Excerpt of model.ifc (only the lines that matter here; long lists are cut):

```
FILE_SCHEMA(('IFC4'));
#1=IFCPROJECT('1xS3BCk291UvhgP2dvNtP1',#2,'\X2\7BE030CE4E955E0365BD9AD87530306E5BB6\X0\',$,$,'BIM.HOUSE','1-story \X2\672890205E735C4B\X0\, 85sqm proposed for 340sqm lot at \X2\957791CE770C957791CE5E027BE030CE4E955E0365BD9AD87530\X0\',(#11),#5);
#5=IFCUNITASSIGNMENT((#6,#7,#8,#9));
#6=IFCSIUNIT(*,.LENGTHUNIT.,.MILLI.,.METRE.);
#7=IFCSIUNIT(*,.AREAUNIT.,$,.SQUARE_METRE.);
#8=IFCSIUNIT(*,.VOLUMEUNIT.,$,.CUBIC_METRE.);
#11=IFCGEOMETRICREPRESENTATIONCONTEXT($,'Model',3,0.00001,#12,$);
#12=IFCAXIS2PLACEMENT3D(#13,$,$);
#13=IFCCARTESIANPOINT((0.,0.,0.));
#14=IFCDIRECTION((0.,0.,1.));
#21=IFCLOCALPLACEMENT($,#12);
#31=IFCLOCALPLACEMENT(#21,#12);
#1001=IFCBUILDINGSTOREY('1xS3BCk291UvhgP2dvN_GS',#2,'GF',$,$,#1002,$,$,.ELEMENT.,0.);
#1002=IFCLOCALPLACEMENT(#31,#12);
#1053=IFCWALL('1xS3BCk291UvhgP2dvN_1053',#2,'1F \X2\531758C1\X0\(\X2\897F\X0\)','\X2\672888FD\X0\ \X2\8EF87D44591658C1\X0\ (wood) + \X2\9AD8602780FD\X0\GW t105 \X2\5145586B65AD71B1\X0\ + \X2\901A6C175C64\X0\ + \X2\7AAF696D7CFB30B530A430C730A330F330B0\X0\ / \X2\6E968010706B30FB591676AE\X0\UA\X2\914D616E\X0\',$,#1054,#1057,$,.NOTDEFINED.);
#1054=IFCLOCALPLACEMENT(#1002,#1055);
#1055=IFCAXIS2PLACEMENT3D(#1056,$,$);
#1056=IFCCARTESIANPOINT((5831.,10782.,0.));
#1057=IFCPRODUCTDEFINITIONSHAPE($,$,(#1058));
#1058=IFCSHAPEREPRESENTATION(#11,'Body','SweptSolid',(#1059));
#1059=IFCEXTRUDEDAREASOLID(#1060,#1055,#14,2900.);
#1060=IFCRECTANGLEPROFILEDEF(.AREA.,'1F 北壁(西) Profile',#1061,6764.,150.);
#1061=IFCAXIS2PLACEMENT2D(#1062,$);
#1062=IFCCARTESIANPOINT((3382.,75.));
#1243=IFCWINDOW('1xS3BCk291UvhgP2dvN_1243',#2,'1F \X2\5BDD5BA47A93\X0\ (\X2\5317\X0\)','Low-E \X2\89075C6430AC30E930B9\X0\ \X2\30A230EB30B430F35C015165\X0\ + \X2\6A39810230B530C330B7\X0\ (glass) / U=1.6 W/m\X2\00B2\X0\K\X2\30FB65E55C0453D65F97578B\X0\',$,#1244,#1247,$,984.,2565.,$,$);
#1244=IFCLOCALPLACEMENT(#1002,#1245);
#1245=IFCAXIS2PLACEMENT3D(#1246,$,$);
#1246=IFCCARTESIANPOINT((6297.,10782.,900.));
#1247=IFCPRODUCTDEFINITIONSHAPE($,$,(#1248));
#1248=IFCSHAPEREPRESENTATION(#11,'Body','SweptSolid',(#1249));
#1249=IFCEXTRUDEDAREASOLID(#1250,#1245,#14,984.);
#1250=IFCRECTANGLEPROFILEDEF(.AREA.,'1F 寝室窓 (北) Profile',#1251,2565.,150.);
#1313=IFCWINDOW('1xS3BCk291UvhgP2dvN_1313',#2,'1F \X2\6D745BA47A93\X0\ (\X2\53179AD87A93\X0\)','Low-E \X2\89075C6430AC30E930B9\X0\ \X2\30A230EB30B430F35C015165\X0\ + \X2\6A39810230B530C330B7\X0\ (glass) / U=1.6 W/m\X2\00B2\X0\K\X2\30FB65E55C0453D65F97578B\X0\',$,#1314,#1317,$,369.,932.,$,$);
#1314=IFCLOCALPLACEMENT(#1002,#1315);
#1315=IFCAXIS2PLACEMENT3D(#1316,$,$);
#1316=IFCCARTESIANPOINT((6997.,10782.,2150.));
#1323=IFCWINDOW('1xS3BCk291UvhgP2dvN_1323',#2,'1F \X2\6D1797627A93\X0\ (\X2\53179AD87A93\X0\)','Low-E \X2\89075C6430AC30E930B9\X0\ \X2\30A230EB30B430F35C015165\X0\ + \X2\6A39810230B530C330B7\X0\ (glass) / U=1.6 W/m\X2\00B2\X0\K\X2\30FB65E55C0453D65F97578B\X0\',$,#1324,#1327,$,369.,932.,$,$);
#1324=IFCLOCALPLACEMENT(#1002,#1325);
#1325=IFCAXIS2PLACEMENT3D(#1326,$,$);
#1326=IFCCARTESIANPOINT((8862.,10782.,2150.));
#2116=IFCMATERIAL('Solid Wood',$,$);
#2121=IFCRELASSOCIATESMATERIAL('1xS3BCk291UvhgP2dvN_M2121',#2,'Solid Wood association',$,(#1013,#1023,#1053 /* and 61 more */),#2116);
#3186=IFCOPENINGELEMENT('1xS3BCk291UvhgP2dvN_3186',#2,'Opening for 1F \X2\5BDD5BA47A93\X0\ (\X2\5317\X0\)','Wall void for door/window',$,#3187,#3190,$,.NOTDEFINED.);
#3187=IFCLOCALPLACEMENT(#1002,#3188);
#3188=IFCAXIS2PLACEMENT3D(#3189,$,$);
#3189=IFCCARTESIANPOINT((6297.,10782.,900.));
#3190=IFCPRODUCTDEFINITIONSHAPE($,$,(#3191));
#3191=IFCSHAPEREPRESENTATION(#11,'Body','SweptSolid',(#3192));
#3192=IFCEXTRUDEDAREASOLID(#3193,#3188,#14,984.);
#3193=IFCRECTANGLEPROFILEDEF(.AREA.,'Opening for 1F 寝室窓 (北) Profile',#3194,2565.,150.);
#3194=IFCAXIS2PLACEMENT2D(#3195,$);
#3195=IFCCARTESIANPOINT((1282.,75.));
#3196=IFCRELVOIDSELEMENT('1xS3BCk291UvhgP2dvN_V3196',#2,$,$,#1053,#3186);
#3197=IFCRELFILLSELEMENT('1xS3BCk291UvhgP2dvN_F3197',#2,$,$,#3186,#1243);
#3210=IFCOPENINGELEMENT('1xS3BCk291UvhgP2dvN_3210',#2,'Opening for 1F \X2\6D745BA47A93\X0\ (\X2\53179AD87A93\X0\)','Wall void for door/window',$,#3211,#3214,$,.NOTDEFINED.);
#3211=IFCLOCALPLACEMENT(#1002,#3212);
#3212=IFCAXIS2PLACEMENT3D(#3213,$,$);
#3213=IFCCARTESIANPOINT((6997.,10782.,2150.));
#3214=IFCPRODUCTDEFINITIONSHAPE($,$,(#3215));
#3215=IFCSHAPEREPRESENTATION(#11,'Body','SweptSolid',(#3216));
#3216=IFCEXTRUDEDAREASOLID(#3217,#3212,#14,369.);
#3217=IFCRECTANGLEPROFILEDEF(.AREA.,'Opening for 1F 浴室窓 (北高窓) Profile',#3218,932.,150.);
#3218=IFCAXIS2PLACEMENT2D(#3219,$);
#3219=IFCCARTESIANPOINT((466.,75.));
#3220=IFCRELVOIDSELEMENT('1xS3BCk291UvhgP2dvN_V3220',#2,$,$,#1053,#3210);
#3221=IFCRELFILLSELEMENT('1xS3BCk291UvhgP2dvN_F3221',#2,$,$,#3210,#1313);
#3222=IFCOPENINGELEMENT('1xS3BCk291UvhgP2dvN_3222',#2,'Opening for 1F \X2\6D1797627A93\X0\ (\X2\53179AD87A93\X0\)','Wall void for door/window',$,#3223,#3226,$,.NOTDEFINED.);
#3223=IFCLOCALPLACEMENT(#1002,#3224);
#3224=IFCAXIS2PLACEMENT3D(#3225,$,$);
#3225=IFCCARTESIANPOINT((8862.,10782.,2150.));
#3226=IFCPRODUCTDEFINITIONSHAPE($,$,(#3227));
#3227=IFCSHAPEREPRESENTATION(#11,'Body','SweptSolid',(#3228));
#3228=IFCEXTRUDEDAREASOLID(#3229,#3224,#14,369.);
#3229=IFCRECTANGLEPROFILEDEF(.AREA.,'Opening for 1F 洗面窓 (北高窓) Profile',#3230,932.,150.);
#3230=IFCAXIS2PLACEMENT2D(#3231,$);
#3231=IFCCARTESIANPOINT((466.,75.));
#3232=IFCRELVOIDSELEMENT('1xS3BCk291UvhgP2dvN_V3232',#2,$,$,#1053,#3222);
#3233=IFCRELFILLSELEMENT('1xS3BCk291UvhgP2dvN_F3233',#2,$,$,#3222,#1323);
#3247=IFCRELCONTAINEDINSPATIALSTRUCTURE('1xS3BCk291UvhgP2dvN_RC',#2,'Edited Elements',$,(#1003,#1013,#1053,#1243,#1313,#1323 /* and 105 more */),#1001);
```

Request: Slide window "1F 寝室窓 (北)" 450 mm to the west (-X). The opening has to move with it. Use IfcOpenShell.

```python
import ifcopenshell
import ifcopenshell.api.geometry
import ifcopenshell.util.placement
import ifcopenshell.util.unit

model = ifcopenshell.open("model.ifc")
unit_scale = ifcopenshell.util.unit.calculate_unit_scale(model)

window = model.by_guid("1xS3BCk291UvhgP2dvN_1243")
opening = window.FillsVoids[0].RelatingOpeningElement
wall = opening.VoidsElements[0].RelatingBuildingElement

wall_matrix = ifcopenshell.util.placement.get_local_placement(wall.ObjectPlacement)
shift = wall_matrix[:3, 0] * -0.45 / unit_scale
before = ifcopenshell.util.placement.get_local_placement(window.ObjectPlacement)[:3, 3].copy()

# The window is not placed relative to its opening, so move both.
for product in (opening, window):
    matrix = ifcopenshell.util.placement.get_local_placement(product.ObjectPlacement)
    matrix[:3, 3] += shift
    ifcopenshell.api.geometry.edit_object_placement(model, product=product, matrix=matrix, is_si=False)

after = ifcopenshell.util.placement.get_local_placement(window.ObjectPlacement)[:3, 3]
print("window moved by", (after - before).round(3) + 0.0)

model.write("model_rev.ifc")
```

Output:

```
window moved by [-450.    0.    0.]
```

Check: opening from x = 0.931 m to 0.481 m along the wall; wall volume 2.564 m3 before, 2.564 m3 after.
